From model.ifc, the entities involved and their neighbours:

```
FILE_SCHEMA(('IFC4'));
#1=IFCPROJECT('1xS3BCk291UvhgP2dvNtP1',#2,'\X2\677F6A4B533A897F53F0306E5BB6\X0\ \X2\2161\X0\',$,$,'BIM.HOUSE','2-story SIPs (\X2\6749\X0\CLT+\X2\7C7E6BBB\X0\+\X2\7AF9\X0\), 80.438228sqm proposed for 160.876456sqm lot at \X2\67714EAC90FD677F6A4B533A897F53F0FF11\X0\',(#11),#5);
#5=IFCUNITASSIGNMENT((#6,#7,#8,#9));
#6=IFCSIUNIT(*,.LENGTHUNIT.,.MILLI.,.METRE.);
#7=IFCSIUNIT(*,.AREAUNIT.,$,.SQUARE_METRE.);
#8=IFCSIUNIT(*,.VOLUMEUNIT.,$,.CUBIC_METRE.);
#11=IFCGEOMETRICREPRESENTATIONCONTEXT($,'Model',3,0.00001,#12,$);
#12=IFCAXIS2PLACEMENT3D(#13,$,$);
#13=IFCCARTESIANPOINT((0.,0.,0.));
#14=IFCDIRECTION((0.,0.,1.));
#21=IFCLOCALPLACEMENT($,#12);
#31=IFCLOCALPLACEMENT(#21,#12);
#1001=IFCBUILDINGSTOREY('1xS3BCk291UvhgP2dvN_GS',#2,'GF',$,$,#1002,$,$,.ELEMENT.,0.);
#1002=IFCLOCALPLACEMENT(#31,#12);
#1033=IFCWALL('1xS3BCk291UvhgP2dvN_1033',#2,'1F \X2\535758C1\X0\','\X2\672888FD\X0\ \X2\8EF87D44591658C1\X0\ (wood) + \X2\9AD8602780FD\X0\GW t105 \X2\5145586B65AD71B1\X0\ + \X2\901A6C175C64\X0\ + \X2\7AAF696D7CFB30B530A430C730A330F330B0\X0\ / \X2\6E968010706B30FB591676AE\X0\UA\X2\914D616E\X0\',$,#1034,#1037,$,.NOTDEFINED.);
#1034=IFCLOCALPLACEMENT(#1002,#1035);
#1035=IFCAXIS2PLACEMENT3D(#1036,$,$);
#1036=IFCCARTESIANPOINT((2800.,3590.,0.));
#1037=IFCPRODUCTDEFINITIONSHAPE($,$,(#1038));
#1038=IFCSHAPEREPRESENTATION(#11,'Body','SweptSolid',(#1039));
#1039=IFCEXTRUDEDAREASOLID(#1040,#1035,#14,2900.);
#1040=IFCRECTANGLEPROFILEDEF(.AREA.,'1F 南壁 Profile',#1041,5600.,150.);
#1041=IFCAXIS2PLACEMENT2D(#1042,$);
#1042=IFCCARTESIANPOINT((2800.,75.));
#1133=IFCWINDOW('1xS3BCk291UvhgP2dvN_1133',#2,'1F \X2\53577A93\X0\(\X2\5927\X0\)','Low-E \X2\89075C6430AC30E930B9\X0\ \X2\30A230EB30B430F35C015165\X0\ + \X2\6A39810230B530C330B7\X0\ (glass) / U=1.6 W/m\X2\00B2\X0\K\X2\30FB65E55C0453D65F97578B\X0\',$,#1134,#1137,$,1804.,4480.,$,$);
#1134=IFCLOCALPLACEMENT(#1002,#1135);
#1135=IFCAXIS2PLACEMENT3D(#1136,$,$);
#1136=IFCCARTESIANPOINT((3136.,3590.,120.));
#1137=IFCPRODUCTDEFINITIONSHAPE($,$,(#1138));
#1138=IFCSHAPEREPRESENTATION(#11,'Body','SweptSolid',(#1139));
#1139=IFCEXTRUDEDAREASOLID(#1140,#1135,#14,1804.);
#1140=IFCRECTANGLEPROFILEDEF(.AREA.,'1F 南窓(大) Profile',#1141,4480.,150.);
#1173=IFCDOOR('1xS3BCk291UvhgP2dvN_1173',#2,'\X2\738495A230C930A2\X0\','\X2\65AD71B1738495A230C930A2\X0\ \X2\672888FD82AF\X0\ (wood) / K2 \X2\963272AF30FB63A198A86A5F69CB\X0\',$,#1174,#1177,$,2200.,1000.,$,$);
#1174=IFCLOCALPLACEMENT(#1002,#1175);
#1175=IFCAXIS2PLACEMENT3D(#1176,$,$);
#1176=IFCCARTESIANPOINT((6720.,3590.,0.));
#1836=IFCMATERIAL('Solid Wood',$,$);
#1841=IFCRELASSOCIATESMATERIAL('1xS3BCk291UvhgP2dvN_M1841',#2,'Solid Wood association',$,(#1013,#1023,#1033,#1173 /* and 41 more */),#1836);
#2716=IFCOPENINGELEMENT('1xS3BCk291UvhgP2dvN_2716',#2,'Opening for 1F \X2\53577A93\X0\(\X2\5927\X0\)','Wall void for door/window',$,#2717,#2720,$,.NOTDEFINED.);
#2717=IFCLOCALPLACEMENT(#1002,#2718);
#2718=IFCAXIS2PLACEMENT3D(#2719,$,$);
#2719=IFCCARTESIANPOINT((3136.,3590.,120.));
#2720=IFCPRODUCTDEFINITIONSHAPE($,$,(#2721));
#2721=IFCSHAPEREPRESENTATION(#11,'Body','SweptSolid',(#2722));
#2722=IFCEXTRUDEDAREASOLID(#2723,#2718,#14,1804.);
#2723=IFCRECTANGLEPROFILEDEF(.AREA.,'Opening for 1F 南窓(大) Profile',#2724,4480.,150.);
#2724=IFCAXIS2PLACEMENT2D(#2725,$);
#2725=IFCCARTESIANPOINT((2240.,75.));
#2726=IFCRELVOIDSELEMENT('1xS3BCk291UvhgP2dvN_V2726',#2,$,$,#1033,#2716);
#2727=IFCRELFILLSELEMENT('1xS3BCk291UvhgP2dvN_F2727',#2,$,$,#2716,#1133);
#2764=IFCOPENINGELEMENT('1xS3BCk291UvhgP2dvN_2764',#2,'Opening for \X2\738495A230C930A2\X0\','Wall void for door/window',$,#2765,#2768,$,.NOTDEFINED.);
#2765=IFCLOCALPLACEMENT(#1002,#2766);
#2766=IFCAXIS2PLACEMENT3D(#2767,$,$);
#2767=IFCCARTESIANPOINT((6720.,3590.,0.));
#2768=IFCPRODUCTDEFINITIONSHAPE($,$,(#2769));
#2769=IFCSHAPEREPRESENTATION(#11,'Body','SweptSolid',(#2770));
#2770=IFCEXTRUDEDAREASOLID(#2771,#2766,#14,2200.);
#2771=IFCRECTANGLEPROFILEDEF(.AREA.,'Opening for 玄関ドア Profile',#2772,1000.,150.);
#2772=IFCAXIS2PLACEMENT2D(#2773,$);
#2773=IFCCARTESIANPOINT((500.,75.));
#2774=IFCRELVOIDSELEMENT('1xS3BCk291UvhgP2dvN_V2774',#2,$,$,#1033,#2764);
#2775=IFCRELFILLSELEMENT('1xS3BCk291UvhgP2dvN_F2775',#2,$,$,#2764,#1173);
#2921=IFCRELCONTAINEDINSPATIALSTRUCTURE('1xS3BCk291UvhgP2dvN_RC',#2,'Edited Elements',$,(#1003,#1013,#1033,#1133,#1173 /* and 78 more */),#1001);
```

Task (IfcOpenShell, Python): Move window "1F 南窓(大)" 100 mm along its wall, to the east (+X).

```python
import ifcopenshell
import ifcopenshell.api.geometry
import ifcopenshell.util.placement
import ifcopenshell.util.unit

model = ifcopenshell.open("model.ifc")
unit_scale = ifcopenshell.util.unit.calculate_unit_scale(model)

window = model.by_id(1133)
opening = window.FillsVoids[0].RelatingOpeningElement
wall = opening.VoidsElements[0].RelatingBuildingElement

wall_matrix = ifcopenshell.util.placement.get_local_placement(wall.ObjectPlacement)
shift = wall_matrix[:3, 0] * 0.1 / unit_scale
before = ifcopenshell.util.placement.get_local_placement(window.ObjectPlacement)[:3, 3].copy()

# The window is not placed relative to its opening, so move both.
for product in (opening, window):
    matrix = ifcopenshell.util.placement.get_local_placement(product.ObjectPlacement)
    matrix[:3, 3] += shift
    ifcopenshell.api.geometry.edit_object_placement(model, product=product, matrix=matrix, is_si=False)

after = ifcopenshell.util.placement.get_local_placement(window.ObjectPlacement)[:3, 3]
print("window moved by", (after - before).round(3) + 0.0)

model.write("model_v2.ifc")
```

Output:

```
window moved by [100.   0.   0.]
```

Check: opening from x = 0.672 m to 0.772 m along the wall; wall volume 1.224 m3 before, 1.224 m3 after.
